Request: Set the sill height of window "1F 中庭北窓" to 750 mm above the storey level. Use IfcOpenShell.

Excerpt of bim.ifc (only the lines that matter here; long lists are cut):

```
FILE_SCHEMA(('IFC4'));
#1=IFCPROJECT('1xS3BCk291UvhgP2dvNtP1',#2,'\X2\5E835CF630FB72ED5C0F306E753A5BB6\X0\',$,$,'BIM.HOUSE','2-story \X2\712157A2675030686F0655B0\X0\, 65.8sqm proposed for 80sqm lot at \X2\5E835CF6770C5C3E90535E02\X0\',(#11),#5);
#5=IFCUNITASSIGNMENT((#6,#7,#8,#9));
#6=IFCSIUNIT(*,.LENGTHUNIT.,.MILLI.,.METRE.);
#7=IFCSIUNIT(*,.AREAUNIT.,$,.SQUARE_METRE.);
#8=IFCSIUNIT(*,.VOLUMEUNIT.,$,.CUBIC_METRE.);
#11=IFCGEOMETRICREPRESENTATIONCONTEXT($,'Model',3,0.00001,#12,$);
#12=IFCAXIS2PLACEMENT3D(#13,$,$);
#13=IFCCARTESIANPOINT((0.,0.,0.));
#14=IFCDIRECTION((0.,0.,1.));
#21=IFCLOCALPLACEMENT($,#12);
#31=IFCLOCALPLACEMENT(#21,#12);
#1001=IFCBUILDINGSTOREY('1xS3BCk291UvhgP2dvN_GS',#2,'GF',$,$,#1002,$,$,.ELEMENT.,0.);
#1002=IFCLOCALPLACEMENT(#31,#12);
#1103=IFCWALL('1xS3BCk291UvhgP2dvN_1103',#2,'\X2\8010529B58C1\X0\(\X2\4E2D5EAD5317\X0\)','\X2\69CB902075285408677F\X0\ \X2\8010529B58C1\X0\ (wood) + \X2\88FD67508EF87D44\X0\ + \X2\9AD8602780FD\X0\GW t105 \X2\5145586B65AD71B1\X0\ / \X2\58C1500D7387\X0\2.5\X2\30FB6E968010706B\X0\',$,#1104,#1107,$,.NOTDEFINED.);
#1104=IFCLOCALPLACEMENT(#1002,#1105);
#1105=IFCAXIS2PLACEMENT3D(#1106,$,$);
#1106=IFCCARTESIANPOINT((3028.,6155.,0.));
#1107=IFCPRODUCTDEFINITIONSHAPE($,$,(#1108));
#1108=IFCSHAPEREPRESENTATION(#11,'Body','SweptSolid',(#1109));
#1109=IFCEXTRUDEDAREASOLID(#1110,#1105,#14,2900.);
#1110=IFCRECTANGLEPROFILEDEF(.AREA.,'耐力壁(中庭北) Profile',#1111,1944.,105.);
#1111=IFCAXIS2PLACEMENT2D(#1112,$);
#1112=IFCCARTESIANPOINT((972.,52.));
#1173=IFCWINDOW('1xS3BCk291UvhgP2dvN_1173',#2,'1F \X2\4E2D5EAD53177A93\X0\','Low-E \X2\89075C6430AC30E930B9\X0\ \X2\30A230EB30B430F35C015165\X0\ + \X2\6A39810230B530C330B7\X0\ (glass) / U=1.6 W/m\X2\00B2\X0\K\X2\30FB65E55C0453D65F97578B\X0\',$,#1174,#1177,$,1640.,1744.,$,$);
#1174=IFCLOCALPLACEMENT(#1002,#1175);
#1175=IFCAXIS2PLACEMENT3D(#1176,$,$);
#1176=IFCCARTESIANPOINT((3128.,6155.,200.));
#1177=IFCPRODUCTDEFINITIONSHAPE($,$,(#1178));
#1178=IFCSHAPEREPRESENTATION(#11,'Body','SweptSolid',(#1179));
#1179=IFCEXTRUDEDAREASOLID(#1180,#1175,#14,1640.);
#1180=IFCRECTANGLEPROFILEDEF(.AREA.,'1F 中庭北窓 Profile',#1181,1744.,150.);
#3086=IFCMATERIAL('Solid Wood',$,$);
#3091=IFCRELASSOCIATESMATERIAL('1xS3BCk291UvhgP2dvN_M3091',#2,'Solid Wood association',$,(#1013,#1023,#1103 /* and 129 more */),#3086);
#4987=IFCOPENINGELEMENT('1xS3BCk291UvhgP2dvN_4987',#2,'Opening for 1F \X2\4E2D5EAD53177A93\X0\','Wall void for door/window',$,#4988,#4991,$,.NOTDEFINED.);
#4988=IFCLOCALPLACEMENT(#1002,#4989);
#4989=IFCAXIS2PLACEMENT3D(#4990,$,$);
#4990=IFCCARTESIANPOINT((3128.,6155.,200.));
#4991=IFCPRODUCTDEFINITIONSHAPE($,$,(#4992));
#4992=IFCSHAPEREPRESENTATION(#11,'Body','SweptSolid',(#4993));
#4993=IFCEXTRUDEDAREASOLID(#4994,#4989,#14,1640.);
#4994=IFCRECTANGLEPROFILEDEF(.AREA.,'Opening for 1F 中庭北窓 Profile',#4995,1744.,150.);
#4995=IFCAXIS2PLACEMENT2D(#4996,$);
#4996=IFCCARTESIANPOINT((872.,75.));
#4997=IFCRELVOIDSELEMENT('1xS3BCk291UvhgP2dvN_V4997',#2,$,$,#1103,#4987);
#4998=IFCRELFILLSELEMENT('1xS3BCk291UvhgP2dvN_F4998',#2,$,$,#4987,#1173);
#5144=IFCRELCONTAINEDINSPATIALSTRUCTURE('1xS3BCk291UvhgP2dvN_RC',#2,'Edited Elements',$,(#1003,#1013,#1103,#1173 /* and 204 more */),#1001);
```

```python
import numpy as np
import ifcopenshell
import ifcopenshell.api.geometry
import ifcopenshell.geom
import ifcopenshell.util.element
import ifcopenshell.util.placement
import ifcopenshell.util.shape
import ifcopenshell.util.unit

model = ifcopenshell.open("bim.ifc")
unit_scale = ifcopenshell.util.unit.calculate_unit_scale(model)

window = model.by_guid("1xS3BCk291UvhgP2dvN_1173")
opening = window.FillsVoids[0].RelatingOpeningElement
storey = ifcopenshell.util.element.get_container(window, ifc_class="IfcBuildingStorey")
level = ifcopenshell.util.placement.get_local_placement(storey.ObjectPlacement)[2, 3]

# The opening's origin need not be at the sill, so measure its lowest point.
shape = ifcopenshell.geom.create_shape(ifcopenshell.geom.settings(), opening)
bottom = ifcopenshell.util.shape.get_shape_bottom_elevation(shape, shape.geometry) / unit_scale
dz = level + 750.0 - bottom

shift = np.array([0.0, 0.0, dz])
# The window is not placed relative to its opening, so move both.
for product in (opening, window):
    matrix = ifcopenshell.util.placement.get_local_placement(product.ObjectPlacement)
    matrix[:3, 3] += shift
    ifcopenshell.api.geometry.edit_object_placement(model, product=product, matrix=matrix, is_si=False)

print(f"moved by {dz * unit_scale:+.3f} m")

model.write("bim_v2.ifc")
```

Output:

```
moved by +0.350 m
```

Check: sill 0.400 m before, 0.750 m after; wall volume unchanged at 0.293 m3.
